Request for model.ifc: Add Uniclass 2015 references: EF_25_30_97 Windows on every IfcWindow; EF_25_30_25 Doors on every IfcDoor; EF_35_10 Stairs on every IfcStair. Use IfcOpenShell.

First a look at what the model holds.

```python
import ifcopenshell

model = ifcopenshell.open("model.ifc")
print(model.schema)
print("classifications:", [c.Name for c in model.by_type("IfcClassification")])
for ifc_class in ("IfcDoor", "IfcRoof", "IfcStair", "IfcWall", "IfcWindow"):
    print(ifc_class, len(model.by_type(ifc_class)))
```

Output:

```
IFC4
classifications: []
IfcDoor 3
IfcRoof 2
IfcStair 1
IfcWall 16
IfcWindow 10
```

```python
import ifcopenshell
import ifcopenshell.api.classification

model = ifcopenshell.open("model.ifc")

system = ifcopenshell.api.classification.add_classification(model, classification="Uniclass 2015")

codes = {
    "IfcWindow": ("EF_25_30_97", "Windows"),
    "IfcDoor": ("EF_25_30_25", "Doors"),
    "IfcStair": ("EF_35_10", "Stairs"),
}
for ifc_class, (code, name) in codes.items():
    products = model.by_type(ifc_class)
    ifcopenshell.api.classification.add_reference(
        model, products=products, classification=system, identification=code, name=name
    )
    print(code, len(products))

model.write("model-out.ifc")
```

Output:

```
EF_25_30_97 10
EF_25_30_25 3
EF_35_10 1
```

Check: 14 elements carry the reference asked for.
